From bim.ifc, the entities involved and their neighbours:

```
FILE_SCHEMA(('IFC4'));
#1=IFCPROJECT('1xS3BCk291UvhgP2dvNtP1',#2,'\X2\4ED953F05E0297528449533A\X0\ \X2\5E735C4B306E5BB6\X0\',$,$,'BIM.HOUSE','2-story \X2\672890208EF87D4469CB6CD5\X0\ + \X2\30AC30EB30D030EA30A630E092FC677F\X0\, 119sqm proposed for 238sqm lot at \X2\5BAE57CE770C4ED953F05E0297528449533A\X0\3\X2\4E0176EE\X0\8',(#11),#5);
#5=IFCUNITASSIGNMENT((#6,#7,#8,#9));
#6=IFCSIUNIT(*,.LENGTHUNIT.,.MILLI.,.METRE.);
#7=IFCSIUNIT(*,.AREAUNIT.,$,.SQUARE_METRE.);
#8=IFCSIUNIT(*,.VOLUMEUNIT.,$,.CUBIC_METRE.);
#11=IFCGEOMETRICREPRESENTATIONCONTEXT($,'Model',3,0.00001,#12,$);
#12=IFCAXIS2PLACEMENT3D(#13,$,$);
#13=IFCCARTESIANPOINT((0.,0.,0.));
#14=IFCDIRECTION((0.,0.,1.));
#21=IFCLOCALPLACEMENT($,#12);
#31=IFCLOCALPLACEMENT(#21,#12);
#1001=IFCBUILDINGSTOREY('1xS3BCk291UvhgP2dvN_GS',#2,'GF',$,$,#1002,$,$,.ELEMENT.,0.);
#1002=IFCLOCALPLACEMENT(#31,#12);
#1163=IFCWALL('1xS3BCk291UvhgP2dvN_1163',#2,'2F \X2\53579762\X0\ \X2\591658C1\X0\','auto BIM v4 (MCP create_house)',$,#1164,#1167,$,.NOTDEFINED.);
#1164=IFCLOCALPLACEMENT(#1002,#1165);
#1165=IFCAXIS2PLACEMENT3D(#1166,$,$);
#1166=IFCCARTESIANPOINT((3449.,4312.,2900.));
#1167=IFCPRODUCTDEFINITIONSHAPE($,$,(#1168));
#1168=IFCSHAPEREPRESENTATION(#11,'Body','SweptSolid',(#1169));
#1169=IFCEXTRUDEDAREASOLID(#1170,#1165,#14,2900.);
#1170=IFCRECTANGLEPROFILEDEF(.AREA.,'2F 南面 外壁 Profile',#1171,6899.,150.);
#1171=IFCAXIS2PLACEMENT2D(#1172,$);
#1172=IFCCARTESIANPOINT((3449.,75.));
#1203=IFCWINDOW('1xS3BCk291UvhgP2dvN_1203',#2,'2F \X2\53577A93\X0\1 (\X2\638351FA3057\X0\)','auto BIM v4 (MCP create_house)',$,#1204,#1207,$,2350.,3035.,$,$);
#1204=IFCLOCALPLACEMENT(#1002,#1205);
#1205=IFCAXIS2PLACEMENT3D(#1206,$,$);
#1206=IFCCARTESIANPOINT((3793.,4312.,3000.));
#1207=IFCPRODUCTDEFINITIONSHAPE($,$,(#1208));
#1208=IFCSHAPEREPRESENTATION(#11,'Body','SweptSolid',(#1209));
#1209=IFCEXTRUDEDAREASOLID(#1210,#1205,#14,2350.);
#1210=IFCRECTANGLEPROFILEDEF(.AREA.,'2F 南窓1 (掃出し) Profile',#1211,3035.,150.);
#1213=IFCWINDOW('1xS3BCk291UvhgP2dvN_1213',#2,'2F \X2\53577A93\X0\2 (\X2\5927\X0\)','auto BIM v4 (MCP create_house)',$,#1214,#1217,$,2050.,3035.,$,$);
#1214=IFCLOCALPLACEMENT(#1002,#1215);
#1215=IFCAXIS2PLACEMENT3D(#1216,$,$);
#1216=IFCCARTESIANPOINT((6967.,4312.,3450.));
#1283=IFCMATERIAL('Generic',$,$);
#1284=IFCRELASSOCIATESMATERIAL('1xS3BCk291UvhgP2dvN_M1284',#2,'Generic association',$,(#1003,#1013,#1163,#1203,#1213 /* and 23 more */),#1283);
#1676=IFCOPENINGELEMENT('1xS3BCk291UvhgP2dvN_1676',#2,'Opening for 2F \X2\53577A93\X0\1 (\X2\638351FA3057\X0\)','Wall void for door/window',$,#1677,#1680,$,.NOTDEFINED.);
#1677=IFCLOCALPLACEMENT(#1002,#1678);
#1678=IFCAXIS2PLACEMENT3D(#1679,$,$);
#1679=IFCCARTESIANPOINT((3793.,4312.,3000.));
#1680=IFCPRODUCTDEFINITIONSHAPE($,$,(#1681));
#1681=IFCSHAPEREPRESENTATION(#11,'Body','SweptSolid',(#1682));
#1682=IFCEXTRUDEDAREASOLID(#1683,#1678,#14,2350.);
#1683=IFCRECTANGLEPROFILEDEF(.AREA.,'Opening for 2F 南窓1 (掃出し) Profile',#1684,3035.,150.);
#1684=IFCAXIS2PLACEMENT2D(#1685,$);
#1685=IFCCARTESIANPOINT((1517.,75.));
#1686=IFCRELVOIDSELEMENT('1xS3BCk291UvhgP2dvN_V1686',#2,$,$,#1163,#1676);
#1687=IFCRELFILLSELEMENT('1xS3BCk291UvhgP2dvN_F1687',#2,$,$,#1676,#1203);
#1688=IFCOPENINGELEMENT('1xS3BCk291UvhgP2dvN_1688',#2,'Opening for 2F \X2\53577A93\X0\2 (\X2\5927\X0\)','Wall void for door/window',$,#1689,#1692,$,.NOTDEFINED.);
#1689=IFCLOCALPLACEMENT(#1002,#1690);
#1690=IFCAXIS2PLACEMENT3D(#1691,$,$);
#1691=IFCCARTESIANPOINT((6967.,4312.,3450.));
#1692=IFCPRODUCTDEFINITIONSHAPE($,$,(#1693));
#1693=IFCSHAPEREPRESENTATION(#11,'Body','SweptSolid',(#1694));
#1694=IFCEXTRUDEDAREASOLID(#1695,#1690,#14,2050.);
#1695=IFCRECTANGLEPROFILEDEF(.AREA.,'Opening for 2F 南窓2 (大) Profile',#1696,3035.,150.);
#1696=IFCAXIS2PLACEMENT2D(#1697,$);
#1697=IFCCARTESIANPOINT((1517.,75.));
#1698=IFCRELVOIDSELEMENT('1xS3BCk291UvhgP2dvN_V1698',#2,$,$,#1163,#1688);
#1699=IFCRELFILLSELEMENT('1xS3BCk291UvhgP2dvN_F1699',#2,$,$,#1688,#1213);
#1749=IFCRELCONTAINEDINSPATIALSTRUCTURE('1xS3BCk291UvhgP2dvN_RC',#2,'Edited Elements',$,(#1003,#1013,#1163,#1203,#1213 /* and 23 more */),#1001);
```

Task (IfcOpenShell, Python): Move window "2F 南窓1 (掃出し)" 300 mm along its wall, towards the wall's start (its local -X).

```python
import ifcopenshell
import ifcopenshell.api.geometry
import ifcopenshell.util.placement
import ifcopenshell.util.unit

model = ifcopenshell.open("bim.ifc")
unit_scale = ifcopenshell.util.unit.calculate_unit_scale(model)

window = model.by_id(1203)
opening = window.FillsVoids[0].RelatingOpeningElement
wall = opening.VoidsElements[0].RelatingBuildingElement

wall_matrix = ifcopenshell.util.placement.get_local_placement(wall.ObjectPlacement)
shift = wall_matrix[:3, 0] * -0.3 / unit_scale
before = ifcopenshell.util.placement.get_local_placement(window.ObjectPlacement)[:3, 3].copy()

# The window is not placed relative to its opening, so move both.
for product in (opening, window):
    matrix = ifcopenshell.util.placement.get_local_placement(product.ObjectPlacement)
    matrix[:3, 3] += shift
    ifcopenshell.api.geometry.edit_object_placement(model, product=product, matrix=matrix, is_si=False)

after = ifcopenshell.util.placement.get_local_placement(window.ObjectPlacement)[:3, 3]
print("window moved by", (after - before).round(3) + 0.0)

model.write("bim_v2.ifc")
```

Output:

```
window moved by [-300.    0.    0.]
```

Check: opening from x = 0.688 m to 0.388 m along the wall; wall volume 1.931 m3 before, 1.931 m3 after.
